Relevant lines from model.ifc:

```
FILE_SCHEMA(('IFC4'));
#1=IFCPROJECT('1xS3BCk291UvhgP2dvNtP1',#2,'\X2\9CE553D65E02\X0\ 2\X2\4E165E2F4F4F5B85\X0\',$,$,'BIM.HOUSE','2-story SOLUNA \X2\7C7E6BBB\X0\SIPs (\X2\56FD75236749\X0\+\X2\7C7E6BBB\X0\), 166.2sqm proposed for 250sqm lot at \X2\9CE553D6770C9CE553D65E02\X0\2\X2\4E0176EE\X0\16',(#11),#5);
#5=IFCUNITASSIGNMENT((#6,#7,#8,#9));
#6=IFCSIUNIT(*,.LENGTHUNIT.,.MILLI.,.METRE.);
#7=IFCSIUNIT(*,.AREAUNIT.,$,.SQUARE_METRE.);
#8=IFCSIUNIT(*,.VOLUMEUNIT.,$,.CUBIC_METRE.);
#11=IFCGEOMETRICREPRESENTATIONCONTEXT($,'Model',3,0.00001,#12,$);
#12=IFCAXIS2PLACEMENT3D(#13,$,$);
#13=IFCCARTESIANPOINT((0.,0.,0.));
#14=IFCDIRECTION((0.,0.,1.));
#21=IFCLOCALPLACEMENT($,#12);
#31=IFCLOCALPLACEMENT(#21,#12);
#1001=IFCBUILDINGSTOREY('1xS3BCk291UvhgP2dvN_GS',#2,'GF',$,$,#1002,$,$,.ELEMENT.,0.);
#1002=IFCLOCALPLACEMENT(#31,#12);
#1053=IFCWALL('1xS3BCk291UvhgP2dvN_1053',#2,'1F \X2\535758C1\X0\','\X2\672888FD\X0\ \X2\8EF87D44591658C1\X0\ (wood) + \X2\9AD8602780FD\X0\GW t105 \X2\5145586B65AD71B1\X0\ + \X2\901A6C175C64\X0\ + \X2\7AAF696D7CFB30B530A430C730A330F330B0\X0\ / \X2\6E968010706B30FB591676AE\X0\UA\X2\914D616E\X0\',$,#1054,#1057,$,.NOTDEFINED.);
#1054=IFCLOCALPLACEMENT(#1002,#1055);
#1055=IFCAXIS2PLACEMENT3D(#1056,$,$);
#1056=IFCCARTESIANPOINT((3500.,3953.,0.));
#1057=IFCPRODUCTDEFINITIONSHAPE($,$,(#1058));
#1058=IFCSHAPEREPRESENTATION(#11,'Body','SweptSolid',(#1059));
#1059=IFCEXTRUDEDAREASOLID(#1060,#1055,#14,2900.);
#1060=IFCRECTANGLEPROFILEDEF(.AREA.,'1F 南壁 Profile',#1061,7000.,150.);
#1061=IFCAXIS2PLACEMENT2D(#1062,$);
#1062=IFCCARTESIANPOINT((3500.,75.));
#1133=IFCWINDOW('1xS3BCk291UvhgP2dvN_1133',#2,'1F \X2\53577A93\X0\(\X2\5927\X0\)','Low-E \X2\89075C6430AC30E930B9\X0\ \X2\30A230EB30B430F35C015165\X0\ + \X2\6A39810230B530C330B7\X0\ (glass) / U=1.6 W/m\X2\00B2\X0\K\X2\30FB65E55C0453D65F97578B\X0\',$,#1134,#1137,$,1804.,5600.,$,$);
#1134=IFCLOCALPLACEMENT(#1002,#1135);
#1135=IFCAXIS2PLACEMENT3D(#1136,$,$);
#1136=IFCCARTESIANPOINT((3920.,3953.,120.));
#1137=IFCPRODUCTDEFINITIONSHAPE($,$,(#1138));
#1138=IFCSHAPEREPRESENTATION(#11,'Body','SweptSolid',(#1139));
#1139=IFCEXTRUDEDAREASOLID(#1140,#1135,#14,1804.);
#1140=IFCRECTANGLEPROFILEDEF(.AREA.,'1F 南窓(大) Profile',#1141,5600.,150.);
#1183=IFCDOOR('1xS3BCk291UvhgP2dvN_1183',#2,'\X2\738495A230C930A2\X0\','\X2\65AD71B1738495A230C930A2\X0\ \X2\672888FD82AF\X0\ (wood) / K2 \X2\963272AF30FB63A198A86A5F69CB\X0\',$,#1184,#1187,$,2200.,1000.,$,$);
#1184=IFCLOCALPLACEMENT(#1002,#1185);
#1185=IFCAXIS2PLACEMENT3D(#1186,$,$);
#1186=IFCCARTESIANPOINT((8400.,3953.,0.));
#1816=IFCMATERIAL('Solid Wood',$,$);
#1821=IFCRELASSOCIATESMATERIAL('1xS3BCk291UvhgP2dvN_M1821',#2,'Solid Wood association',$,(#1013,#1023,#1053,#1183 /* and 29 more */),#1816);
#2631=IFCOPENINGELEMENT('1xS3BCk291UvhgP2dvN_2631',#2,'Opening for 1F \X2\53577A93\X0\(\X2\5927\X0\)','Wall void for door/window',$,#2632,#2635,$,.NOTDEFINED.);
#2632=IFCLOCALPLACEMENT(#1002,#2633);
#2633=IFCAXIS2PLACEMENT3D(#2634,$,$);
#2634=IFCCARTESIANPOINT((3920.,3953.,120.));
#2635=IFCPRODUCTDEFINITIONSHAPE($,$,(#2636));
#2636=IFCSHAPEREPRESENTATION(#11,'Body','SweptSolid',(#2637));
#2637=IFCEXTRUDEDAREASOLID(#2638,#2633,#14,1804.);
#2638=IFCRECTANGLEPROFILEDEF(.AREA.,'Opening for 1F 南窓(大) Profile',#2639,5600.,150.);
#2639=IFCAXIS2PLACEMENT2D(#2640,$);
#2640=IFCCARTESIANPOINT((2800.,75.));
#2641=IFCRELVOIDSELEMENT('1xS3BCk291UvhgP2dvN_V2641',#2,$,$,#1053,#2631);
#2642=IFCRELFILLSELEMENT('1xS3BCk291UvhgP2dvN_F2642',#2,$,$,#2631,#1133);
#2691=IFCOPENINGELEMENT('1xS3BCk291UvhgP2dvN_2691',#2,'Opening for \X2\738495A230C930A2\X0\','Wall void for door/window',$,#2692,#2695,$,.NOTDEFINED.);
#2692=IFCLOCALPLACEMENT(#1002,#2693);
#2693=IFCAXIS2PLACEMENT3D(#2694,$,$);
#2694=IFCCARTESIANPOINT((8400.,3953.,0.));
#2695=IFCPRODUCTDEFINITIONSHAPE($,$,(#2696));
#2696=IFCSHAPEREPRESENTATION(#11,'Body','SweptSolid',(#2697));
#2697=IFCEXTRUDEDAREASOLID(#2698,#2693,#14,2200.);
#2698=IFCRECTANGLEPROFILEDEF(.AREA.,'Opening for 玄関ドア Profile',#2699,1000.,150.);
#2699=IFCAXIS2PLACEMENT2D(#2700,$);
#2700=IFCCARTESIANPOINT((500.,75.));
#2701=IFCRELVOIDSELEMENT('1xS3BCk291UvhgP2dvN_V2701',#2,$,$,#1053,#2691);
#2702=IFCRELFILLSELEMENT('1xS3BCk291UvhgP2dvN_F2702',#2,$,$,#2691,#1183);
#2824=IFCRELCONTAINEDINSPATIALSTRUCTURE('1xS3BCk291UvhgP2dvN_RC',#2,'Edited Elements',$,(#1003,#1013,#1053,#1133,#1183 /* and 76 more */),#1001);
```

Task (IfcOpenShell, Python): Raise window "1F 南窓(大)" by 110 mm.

```python
import numpy as np
import ifcopenshell
import ifcopenshell.api.geometry
import ifcopenshell.util.placement
import ifcopenshell.util.unit

model = ifcopenshell.open("model.ifc")
unit_scale = ifcopenshell.util.unit.calculate_unit_scale(model)

window = model.by_guid("1xS3BCk291UvhgP2dvN_1133")
opening = window.FillsVoids[0].RelatingOpeningElement
dz = 0.11 / unit_scale

shift = np.array([0.0, 0.0, dz])
# The window is not placed relative to its opening, so move both.
for product in (opening, window):
    matrix = ifcopenshell.util.placement.get_local_placement(product.ObjectPlacement)
    matrix[:3, 3] += shift
    ifcopenshell.api.geometry.edit_object_placement(model, product=product, matrix=matrix, is_si=False)

print(f"moved by {dz * unit_scale:+.3f} m")

model.write("model_updated.ifc")
```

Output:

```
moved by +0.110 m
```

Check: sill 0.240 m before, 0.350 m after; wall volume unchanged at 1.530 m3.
